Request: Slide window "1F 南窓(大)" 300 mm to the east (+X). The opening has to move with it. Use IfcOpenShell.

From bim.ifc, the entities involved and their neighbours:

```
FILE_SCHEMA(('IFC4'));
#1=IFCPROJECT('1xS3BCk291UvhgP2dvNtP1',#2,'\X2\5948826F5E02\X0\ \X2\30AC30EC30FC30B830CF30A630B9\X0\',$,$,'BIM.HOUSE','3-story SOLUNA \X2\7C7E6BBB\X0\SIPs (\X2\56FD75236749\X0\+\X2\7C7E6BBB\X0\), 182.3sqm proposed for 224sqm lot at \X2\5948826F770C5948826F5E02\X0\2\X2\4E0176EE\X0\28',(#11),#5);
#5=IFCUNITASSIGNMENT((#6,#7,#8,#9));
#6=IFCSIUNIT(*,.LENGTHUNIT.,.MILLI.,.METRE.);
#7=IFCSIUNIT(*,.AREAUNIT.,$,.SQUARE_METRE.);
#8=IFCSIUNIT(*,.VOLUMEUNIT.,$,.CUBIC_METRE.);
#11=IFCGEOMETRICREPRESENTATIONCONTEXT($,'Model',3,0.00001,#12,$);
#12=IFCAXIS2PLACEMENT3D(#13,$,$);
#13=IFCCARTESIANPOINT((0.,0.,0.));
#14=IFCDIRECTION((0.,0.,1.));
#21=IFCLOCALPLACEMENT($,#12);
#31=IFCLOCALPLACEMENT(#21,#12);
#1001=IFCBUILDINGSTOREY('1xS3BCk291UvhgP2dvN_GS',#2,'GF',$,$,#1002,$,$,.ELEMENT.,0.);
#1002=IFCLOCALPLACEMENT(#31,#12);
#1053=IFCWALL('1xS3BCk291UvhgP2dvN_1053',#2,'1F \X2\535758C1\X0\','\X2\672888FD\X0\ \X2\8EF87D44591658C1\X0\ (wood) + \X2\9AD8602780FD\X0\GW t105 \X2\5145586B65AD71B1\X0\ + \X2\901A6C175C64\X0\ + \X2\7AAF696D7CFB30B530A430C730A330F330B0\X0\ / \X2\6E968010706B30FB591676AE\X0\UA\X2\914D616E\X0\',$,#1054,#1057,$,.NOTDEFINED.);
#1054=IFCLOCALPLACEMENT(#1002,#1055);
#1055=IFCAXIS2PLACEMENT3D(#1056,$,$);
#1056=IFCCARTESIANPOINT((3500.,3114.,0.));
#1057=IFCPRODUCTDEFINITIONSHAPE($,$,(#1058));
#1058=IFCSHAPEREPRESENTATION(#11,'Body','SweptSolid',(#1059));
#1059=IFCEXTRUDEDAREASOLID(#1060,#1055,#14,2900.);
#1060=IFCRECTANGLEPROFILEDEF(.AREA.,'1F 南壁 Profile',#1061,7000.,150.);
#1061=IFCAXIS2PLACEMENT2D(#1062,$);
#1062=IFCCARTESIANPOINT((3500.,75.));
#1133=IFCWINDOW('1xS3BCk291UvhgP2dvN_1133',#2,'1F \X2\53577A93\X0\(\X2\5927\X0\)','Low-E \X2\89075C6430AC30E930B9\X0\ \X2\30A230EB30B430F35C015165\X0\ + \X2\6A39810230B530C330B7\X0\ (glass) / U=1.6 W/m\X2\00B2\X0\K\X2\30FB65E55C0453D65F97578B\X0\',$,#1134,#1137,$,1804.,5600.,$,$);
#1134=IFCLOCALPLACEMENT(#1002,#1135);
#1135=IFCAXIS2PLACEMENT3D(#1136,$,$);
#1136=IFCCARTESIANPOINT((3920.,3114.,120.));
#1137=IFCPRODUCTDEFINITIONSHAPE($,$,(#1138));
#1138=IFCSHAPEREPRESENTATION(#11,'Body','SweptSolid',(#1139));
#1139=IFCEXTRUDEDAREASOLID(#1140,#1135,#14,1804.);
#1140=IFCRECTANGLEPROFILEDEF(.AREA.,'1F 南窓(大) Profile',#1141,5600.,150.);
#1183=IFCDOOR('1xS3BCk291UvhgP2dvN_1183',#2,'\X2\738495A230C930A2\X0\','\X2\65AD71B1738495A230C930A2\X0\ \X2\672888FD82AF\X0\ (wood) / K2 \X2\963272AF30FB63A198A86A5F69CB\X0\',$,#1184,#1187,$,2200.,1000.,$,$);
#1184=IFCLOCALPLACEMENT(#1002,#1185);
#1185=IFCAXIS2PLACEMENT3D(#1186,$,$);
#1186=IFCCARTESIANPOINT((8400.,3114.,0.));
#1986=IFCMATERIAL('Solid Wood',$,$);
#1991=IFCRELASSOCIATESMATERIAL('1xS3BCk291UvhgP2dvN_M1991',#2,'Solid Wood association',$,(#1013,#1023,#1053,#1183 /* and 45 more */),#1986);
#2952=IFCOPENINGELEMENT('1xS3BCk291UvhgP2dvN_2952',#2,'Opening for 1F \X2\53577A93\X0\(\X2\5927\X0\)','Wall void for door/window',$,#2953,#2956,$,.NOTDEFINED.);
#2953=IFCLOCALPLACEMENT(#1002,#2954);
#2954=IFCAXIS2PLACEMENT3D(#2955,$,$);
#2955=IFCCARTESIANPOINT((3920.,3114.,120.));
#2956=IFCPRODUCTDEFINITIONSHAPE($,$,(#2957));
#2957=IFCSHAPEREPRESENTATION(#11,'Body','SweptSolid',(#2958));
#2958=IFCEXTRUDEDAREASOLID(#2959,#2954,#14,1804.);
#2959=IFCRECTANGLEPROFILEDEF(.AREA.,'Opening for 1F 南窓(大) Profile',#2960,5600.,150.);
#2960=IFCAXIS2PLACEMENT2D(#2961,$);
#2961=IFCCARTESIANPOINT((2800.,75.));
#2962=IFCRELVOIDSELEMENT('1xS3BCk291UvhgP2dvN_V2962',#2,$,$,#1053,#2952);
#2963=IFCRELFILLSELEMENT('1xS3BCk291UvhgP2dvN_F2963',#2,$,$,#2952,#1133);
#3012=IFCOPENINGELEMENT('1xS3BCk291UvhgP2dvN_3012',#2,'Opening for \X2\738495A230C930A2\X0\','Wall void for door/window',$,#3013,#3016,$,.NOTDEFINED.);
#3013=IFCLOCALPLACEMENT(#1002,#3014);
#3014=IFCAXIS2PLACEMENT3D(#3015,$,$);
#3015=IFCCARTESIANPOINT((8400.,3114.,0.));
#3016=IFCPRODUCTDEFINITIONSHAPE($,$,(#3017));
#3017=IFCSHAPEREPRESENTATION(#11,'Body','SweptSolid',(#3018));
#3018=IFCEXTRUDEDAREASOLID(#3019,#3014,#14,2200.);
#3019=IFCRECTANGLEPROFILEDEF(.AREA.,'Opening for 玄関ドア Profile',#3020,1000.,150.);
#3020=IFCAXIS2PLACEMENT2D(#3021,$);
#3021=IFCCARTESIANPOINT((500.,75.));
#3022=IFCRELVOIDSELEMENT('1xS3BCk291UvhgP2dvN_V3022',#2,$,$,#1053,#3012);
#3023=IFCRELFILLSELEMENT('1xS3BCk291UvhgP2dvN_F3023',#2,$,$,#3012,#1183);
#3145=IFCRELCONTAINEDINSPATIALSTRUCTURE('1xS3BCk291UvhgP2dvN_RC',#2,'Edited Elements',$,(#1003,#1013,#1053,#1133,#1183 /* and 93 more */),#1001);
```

```python
import ifcopenshell
import ifcopenshell.api.geometry
import ifcopenshell.util.placement

model = ifcopenshell.open("bim.ifc")

window = model.by_guid("1xS3BCk291UvhgP2dvN_1133")
opening = window.FillsVoids[0].RelatingOpeningElement
wall = opening.VoidsElements[0].RelatingBuildingElement

wall_matrix = ifcopenshell.util.placement.get_local_placement(wall.ObjectPlacement)
shift = wall_matrix[:3, 0] * 300.0
before = ifcopenshell.util.placement.get_local_placement(window.ObjectPlacement)[:3, 3].copy()

# The window is not placed relative to its opening, so move both.
for product in (opening, window):
    matrix = ifcopenshell.util.placement.get_local_placement(product.ObjectPlacement)
    matrix[:3, 3] += shift
    ifcopenshell.api.geometry.edit_object_placement(model, product=product, matrix=matrix, is_si=False)

after = ifcopenshell.util.placement.get_local_placement(window.ObjectPlacement)[:3, 3]
print("window moved by", (after - before).round(3) + 0.0)

model.write("bim_rev.ifc")
```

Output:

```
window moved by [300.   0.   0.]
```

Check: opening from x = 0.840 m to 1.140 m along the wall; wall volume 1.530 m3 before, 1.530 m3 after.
